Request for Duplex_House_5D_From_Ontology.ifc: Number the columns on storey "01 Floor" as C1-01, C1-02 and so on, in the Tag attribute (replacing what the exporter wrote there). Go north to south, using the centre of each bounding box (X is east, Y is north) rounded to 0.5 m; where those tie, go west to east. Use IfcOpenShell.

First a look at what the model holds.

```python
import ifcopenshell
import ifcopenshell.util.element
import ifcopenshell.util.placement

model = ifcopenshell.open("Duplex_House_5D_From_Ontology.ifc")
print(model.schema)
storey = next(s for s in model.by_type("IfcBuildingStorey") if s.Name == "01 Floor")
columns = [e for e in ifcopenshell.util.element.get_decomposition(storey) if e.is_a("IfcColumn")]
for e in sorted(columns, key=lambda e: e.id()):
    origin = ifcopenshell.util.placement.get_local_placement(e.ObjectPlacement)[:3, 3]
    print(e.id(), e.Tag, e.Name, origin.round(2) + 0.0, sep=" | ")
```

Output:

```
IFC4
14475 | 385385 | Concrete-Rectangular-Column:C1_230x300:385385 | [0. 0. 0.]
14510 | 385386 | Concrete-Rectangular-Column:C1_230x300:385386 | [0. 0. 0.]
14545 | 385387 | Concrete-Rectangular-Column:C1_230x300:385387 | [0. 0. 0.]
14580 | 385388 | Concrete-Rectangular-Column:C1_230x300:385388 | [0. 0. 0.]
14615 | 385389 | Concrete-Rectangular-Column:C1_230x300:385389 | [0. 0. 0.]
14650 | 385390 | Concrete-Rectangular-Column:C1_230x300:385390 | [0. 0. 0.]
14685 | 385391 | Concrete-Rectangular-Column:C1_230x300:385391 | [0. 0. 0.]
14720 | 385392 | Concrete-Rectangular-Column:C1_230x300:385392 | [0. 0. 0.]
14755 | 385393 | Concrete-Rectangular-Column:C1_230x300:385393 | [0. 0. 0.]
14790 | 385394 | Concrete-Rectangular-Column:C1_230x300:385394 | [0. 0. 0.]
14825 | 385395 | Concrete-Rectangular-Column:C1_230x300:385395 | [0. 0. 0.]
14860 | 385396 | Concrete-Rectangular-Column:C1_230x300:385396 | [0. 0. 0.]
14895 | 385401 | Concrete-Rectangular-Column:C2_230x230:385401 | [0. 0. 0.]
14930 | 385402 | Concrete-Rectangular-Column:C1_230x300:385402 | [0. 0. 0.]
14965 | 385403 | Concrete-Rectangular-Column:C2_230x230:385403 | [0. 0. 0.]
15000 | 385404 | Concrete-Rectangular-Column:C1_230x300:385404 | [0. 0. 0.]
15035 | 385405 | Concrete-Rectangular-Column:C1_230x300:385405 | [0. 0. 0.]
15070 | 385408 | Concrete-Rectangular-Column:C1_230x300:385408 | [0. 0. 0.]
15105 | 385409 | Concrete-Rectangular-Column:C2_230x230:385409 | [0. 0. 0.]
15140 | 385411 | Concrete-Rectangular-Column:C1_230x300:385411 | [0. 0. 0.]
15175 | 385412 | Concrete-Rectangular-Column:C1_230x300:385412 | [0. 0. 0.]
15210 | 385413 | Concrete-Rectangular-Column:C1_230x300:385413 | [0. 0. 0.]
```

```python
import ifcopenshell
import ifcopenshell.geom
import ifcopenshell.util.element
import ifcopenshell.util.shape

model = ifcopenshell.open("Duplex_House_5D_From_Ontology.ifc")
settings = ifcopenshell.geom.settings()
settings.set("use-world-coords", True)


def centre(element):
    shape = ifcopenshell.geom.create_shape(settings, element)
    return ifcopenshell.util.shape.get_bbox_centroid(shape.geometry)


storey = next(s for s in model.by_type("IfcBuildingStorey") if s.Name == "01 Floor")
columns = [e for e in ifcopenshell.util.element.get_decomposition(storey) if e.is_a("IfcColumn")]

# Insertion points can sit at a corner or the storey origin, so sort by the geometry (in metres).
centres = {e: centre(e) for e in columns}
columns.sort(key=lambda e: (-round(centres[e][1] / 0.5), centres[e][0]))

for i, e in enumerate(columns, start=1):
    number = f"C1-{i:02d}"
    e.Tag = number
    print(e.id(), number)

model.write("Duplex_House_5D_From_Ontology_rev.ifc")
```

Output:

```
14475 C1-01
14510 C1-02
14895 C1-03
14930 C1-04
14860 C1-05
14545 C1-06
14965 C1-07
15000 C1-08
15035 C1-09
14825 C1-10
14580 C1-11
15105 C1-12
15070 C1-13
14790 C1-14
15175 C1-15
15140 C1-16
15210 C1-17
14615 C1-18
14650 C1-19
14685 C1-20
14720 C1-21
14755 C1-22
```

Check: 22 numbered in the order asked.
